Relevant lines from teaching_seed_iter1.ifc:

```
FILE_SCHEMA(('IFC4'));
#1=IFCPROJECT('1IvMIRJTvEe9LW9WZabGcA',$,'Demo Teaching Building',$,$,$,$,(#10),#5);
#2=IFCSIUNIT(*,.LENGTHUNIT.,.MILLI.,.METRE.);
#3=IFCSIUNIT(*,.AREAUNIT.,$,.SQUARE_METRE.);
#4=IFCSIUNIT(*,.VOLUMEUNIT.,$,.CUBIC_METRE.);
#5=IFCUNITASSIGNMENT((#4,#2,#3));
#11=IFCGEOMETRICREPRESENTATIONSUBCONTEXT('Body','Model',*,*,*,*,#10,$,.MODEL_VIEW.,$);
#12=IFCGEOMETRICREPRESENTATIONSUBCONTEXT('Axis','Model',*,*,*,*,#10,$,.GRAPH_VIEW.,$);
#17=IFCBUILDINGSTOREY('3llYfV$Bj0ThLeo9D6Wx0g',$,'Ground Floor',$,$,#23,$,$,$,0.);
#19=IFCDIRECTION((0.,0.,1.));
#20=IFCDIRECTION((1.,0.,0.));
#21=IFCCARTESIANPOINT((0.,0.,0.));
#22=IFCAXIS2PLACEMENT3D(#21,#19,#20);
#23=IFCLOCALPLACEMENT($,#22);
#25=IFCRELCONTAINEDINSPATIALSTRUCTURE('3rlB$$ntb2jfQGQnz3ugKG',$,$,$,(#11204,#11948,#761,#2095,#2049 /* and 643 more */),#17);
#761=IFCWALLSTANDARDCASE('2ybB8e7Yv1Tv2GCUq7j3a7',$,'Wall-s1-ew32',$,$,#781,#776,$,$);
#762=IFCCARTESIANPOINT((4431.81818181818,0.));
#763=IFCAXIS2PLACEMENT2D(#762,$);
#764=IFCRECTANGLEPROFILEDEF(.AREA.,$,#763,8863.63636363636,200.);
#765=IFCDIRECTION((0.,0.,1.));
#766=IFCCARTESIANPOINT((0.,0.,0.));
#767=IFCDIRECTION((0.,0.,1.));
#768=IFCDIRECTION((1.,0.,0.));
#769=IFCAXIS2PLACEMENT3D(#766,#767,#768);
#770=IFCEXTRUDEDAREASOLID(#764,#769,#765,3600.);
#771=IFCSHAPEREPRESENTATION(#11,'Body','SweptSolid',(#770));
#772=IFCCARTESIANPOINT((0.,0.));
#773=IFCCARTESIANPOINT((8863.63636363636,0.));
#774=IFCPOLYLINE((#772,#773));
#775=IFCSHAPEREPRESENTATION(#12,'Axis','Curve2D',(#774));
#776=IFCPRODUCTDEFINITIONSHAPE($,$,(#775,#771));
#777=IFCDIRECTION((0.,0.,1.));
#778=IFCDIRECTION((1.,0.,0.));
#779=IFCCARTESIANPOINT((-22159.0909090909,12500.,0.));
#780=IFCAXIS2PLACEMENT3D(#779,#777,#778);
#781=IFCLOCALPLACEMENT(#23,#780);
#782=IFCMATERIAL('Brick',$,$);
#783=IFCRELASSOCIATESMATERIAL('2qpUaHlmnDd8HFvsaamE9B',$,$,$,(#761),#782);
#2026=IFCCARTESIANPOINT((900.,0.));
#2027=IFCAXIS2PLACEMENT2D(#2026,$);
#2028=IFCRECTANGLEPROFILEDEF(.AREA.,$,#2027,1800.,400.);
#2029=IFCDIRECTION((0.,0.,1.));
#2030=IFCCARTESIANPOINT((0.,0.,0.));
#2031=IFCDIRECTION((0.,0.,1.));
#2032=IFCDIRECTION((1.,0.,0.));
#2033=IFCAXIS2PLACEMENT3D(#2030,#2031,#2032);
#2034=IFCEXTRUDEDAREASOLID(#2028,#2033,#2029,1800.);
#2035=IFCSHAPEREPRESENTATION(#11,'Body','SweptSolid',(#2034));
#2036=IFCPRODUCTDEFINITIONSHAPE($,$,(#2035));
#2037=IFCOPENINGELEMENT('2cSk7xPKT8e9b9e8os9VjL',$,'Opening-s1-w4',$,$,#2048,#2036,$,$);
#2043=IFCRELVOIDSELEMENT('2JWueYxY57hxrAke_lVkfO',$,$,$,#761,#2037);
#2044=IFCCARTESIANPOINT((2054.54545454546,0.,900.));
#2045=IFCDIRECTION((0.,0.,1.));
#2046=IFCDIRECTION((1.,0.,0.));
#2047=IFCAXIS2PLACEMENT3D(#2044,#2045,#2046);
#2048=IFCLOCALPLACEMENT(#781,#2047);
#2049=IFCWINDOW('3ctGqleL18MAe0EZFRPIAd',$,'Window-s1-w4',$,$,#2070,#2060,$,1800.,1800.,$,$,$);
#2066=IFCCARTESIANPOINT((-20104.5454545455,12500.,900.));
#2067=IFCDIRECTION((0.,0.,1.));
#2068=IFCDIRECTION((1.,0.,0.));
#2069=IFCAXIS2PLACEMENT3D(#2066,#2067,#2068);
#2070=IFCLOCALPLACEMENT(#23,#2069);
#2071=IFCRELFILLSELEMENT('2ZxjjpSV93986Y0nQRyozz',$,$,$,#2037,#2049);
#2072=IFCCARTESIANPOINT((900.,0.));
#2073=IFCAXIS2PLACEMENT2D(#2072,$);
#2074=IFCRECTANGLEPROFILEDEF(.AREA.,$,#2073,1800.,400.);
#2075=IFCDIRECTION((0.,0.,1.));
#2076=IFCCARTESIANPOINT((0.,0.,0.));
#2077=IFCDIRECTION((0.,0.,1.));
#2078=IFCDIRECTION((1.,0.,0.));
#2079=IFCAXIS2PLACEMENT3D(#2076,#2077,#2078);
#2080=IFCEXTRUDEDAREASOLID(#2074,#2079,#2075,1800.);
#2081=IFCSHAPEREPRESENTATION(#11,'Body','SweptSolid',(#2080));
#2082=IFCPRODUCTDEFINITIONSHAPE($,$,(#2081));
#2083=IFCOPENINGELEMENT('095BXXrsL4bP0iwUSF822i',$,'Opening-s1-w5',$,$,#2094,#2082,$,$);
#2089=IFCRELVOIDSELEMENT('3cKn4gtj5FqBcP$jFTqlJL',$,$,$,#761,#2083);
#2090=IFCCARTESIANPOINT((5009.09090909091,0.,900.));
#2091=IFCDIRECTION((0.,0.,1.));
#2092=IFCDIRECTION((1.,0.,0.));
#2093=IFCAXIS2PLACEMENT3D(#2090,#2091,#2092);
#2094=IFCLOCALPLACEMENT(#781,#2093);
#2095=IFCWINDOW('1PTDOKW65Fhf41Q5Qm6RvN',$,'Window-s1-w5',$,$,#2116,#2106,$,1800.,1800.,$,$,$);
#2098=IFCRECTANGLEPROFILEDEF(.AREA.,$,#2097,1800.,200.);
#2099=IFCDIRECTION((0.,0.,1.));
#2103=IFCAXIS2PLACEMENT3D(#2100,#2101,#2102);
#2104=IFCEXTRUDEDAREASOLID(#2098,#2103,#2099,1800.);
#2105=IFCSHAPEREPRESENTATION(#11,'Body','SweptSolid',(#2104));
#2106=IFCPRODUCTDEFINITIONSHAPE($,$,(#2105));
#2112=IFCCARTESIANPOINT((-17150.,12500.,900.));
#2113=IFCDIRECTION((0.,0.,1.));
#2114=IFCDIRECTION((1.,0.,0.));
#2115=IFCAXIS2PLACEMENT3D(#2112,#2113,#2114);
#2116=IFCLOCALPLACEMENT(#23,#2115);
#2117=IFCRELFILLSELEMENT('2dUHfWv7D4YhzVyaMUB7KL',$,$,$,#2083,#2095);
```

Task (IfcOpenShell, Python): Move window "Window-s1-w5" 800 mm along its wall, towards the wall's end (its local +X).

```python
import ifcopenshell
import ifcopenshell.api.geometry
import ifcopenshell.util.placement
import ifcopenshell.util.unit

model = ifcopenshell.open("teaching_seed_iter1.ifc")
unit_scale = ifcopenshell.util.unit.calculate_unit_scale(model)

window = model.by_guid("1PTDOKW65Fhf41Q5Qm6RvN")
opening = window.FillsVoids[0].RelatingOpeningElement
wall = opening.VoidsElements[0].RelatingBuildingElement

wall_matrix = ifcopenshell.util.placement.get_local_placement(wall.ObjectPlacement)
shift = wall_matrix[:3, 0] * 0.8 / unit_scale
before = ifcopenshell.util.placement.get_local_placement(window.ObjectPlacement)[:3, 3].copy()

# The window is not placed relative to its opening, so move both.
for product in (opening, window):
    matrix = ifcopenshell.util.placement.get_local_placement(product.ObjectPlacement)
    matrix[:3, 3] += shift
    ifcopenshell.api.geometry.edit_object_placement(model, product=product, matrix=matrix, is_si=False)

after = ifcopenshell.util.placement.get_local_placement(window.ObjectPlacement)[:3, 3]
print("window moved by", (after - before).round(3) + 0.0)

model.write("teaching_seed_iter1_v2.ifc")
```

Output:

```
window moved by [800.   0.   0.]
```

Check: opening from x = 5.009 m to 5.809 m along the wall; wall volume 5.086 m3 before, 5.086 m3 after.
